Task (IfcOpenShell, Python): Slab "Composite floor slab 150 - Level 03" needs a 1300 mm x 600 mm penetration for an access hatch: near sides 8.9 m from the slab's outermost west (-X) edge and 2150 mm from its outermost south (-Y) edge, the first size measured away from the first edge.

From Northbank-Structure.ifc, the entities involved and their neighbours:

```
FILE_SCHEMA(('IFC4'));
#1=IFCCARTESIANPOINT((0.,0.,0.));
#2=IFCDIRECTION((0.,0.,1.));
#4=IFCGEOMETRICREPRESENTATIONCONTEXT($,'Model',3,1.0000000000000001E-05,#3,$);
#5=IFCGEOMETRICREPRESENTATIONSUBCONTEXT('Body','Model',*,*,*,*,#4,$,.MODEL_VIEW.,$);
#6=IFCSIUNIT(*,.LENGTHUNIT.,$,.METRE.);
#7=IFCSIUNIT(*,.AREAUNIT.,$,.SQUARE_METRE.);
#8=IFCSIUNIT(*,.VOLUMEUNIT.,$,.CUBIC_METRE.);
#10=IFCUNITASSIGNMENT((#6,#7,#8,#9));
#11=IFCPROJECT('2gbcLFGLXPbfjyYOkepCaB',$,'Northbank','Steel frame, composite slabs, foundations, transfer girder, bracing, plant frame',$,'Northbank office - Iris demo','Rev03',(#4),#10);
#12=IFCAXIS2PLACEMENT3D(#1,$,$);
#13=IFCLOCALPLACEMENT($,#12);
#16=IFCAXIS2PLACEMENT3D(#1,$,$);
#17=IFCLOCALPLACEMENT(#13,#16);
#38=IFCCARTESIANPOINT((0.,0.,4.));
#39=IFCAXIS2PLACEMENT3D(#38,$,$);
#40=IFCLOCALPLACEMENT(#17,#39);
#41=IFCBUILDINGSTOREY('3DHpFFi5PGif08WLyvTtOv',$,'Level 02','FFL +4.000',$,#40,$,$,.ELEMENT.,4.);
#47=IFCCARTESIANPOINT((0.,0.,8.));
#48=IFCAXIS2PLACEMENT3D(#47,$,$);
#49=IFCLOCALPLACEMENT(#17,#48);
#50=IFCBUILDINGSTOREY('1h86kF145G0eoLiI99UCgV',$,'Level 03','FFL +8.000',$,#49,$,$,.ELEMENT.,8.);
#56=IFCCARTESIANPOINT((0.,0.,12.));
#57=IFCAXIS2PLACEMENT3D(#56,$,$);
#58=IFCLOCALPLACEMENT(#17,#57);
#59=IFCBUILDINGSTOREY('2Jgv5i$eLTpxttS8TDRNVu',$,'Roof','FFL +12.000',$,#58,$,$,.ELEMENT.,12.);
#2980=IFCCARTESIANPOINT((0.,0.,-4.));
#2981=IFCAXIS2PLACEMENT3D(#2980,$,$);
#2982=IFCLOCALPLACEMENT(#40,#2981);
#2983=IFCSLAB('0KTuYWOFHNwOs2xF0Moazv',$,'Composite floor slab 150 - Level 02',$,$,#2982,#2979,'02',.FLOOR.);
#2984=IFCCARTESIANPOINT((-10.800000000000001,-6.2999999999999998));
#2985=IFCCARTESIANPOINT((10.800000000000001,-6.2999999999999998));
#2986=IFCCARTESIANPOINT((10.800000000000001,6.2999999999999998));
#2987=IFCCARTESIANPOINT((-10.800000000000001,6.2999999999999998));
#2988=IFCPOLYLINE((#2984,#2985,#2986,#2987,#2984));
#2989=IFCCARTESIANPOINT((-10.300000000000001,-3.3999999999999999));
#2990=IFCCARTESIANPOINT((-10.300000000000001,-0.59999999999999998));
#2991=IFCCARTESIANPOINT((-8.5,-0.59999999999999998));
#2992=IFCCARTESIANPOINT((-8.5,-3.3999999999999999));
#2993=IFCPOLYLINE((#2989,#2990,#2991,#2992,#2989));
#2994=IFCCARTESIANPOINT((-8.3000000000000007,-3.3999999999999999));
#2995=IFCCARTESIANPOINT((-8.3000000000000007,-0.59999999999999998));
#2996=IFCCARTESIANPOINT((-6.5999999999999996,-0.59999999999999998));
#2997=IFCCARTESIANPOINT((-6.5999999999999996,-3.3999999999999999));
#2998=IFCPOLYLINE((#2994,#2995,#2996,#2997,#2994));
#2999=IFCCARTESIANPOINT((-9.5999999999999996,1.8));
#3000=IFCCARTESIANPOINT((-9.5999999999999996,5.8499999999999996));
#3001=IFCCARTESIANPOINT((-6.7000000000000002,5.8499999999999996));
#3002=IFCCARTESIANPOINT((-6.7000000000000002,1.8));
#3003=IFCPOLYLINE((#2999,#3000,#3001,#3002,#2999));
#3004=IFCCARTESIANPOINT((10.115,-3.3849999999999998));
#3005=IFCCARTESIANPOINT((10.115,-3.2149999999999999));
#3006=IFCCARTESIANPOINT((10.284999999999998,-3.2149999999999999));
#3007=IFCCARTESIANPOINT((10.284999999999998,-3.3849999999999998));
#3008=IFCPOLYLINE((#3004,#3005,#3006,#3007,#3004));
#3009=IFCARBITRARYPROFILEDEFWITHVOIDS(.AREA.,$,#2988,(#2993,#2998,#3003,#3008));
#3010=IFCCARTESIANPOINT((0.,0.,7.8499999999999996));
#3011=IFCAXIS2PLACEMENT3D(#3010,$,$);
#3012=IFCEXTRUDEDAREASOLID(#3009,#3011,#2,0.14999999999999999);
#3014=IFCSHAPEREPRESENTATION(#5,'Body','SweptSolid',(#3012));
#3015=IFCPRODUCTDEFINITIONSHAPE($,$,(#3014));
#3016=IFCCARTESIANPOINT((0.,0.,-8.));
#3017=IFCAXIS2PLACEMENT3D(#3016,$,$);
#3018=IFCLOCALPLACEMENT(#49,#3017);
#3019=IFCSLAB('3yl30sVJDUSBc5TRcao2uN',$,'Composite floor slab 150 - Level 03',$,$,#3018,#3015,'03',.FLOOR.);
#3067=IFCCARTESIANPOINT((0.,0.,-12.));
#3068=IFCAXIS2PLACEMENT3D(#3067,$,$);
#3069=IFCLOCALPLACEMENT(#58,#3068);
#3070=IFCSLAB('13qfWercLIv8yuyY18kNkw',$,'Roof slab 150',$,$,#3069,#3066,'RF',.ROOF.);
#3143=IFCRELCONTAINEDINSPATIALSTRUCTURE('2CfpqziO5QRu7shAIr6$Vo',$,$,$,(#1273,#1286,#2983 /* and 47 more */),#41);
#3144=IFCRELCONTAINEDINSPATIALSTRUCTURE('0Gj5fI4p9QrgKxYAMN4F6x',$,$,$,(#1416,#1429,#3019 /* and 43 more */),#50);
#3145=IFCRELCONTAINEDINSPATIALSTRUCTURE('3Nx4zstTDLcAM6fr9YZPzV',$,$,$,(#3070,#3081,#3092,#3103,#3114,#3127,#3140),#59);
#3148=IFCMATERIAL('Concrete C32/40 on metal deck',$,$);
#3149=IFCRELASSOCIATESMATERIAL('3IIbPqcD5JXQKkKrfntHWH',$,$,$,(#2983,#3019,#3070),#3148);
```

```python
import numpy as np
import ifcopenshell
import ifcopenshell.api.feature
import ifcopenshell.api.geometry
import ifcopenshell.api.root
import ifcopenshell.geom
import ifcopenshell.util.placement
import ifcopenshell.util.representation
import ifcopenshell.util.shape
import ifcopenshell.util.unit

model = ifcopenshell.open("Northbank-Structure.ifc")
unit_scale = ifcopenshell.util.unit.calculate_unit_scale(model)
settings = ifcopenshell.geom.settings()


def volume(element):
    """Net volume in cubic metres, openings subtracted."""
    shape = ifcopenshell.geom.create_shape(settings, element)
    return ifcopenshell.util.shape.get_volume(shape.geometry)


slab = model.by_guid("3yl30sVJDUSBc5TRcao2uN")
before = volume(slab)

# Extent in the slab's own axes, in metres. The edges named are its -X and -Y sides.
slab_shape = ifcopenshell.geom.create_shape(settings, slab)
vertices = ifcopenshell.util.shape.get_vertices(slab_shape.geometry)
x_min, y_min, bottom = vertices.min(axis=0)
top = vertices[:, 2].max()

opening = ifcopenshell.api.root.create_entity(model, ifc_class="IfcOpeningElement", name="Access hatch opening", predefined_type="OPENING")
context = ifcopenshell.util.representation.get_context(model, "Model", "Body", "MODEL_VIEW")
width, depth = 1.3, 0.6
outline = [(0.0, 0.0), (width, 0.0), (width, depth), (0.0, depth), (0.0, 0.0)]
# Overshoot both faces by 50 mm so the cut is clean.
shape = ifcopenshell.api.geometry.add_slab_representation(
    model, context=context, depth=top - bottom + 0.1, polyline=outline
)
ifcopenshell.api.geometry.assign_representation(model, product=opening, representation=shape)

matrix = ifcopenshell.util.placement.get_local_placement(slab.ObjectPlacement)
matrix[:, 3] = matrix @ np.append(np.array([x_min + 8.9, y_min + 2.15, bottom - 0.05]) / unit_scale, 1.0)
ifcopenshell.api.geometry.edit_object_placement(model, product=opening, matrix=matrix, is_si=False)
ifcopenshell.api.feature.add_feature(model, feature=opening, element=slab)

after = volume(slab)

print(f"slab volume {before:.3f} -> {after:.3f} m3")

model.write("Northbank-Structure_rev.ifc")
```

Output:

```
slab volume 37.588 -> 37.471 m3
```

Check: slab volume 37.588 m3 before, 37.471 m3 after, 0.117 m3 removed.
